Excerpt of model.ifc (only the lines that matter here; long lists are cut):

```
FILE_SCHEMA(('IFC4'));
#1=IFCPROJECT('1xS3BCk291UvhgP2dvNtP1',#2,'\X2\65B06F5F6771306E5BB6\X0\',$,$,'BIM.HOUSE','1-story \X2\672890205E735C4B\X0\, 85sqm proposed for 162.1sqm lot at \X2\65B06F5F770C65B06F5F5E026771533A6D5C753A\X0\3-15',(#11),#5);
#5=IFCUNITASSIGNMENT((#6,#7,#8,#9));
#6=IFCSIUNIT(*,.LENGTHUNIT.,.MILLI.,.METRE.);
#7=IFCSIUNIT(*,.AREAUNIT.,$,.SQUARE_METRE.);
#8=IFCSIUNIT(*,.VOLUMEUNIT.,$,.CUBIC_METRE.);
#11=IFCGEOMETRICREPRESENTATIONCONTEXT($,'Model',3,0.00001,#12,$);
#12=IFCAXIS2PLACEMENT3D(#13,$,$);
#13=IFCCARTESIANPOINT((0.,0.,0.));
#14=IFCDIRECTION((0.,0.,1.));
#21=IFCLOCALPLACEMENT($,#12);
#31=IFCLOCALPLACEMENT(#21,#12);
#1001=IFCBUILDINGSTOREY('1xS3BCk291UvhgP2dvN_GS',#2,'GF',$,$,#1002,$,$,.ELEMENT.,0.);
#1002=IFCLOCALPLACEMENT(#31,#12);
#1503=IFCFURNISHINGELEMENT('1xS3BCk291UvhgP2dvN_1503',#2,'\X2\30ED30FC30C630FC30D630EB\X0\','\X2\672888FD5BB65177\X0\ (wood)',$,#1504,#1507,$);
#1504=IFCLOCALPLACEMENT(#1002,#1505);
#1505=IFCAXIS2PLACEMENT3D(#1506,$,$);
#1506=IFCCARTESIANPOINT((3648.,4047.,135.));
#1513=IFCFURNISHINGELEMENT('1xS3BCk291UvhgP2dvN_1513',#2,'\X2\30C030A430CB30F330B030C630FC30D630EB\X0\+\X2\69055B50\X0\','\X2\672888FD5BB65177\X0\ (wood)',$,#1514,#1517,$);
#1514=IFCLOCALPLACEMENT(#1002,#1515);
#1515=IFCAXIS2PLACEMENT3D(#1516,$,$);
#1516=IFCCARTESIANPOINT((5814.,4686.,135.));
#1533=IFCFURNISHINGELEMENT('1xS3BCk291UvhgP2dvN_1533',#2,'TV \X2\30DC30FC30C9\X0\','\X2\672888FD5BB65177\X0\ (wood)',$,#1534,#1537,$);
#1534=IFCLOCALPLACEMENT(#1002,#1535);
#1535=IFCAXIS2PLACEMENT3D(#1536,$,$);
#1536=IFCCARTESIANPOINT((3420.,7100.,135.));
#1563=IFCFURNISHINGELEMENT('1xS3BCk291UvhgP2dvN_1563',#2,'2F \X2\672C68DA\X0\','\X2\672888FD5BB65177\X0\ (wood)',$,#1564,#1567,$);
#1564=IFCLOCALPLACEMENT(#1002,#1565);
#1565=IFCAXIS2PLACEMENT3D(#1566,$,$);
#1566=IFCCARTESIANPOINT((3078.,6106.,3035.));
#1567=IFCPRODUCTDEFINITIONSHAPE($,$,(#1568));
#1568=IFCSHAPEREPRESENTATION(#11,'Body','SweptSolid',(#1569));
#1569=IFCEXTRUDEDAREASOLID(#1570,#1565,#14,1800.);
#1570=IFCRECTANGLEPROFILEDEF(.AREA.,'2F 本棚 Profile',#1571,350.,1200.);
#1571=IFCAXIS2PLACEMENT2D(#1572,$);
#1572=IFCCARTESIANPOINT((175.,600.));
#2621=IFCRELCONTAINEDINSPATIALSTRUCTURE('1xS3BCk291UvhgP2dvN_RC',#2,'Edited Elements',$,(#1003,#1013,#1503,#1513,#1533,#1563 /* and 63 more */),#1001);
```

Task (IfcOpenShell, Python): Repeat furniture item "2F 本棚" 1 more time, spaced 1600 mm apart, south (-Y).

```python
import numpy as np
import ifcopenshell
import ifcopenshell.api.geometry
import ifcopenshell.api.root
import ifcopenshell.util.element
import ifcopenshell.util.placement

model = ifcopenshell.open("model.ifc")


def reuse_history(source, copy):
    """copy_class also copies each property set's owner history, people and application; keep the originals."""
    for rel in copy.IsDefinedBy:
        if rel.is_a("IfcRelDefinesByProperties") and (history := rel.RelatingPropertyDefinition.OwnerHistory):
            rel.RelatingPropertyDefinition.OwnerHistory = source.OwnerHistory
            ifcopenshell.util.element.remove_deep2(model, history)


source = model.by_id(1563)
base = ifcopenshell.util.placement.get_local_placement(source.ObjectPlacement)
step = np.array([0.0, -1.0, 0.0]) * 1600.0

for i in range(1, 2):
    copy = ifcopenshell.api.root.copy_class(model, product=source)
    copy.Representation = ifcopenshell.util.element.copy_deep(
        model, source.Representation, exclude=["IfcGeometricRepresentationContext", "IfcRepresentationMap"]
    )
    reuse_history(source, copy)
    matrix = base.copy()
    matrix[:3, 3] += i * step
    print("added at", matrix[:3, 3].round(3) + 0.0)
    ifcopenshell.api.geometry.edit_object_placement(model, product=copy, matrix=matrix, is_si=False)

model.write("model_rev.ifc")
```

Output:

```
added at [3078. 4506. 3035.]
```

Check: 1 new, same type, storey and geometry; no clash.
